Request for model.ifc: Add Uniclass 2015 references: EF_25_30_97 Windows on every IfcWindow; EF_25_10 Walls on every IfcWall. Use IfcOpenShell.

First a look at what the model holds.

```python
import ifcopenshell

model = ifcopenshell.open("model.ifc")
print(model.schema)
print("classifications:", [c.Name for c in model.by_type("IfcClassification")])
for ifc_class in ("IfcDoor", "IfcRoof", "IfcStair", "IfcWall", "IfcWindow"):
    print(ifc_class, len(model.by_type(ifc_class)))
```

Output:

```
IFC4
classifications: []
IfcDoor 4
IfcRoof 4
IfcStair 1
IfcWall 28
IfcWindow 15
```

```python
import ifcopenshell
import ifcopenshell.api.classification

model = ifcopenshell.open("model.ifc")

system = ifcopenshell.api.classification.add_classification(model, classification="Uniclass 2015")

codes = {
    "IfcWindow": ("EF_25_30_97", "Windows"),
    "IfcWall": ("EF_25_10", "Walls"),
}
for ifc_class, (code, name) in codes.items():
    products = model.by_type(ifc_class)
    ifcopenshell.api.classification.add_reference(
        model, products=products, classification=system, identification=code, name=name
    )
    print(code, len(products))

model.write("model_v2.ifc")
```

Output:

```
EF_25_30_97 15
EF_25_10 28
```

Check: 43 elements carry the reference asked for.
